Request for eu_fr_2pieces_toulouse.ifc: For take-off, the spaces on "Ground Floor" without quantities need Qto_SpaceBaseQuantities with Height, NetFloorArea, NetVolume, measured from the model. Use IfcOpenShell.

First a look at what the model holds.

```python
import ifcopenshell
import ifcopenshell.util.element
import ifcopenshell.util.unit

model = ifcopenshell.open("eu_fr_2pieces_toulouse.ifc")
print(model.schema)
for unit_type in ("LENGTHUNIT", "AREAUNIT", "VOLUMEUNIT"):
    print(unit_type, ifcopenshell.util.unit.calculate_unit_scale(model, unit_type))
storey = next(s for s in model.by_type("IfcBuildingStorey") if s.Name == "Ground Floor")
spaces = [e for e in ifcopenshell.util.element.get_decomposition(storey) if e.is_a("IfcSpace")]
for e in sorted(spaces, key=lambda e: e.id()):
    print(e.id(), e.is_a(), e.Name, list(ifcopenshell.util.element.get_psets(e, qtos_only=True)), sep=" | ")
```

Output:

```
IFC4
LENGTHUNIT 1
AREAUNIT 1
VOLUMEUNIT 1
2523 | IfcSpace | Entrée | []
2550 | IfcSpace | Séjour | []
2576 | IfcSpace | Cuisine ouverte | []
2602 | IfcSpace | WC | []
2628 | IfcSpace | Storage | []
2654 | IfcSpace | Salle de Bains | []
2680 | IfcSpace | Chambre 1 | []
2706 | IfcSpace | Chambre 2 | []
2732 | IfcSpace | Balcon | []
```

```python
import ifcopenshell
import ifcopenshell.api.pset
import ifcopenshell.geom
import ifcopenshell.util.element
import ifcopenshell.util.shape
import ifcopenshell.util.unit

model = ifcopenshell.open("eu_fr_2pieces_toulouse.ifc")
unit_scale = ifcopenshell.util.unit.calculate_unit_scale(model)
area_scale = ifcopenshell.util.unit.calculate_unit_scale(model, "AREAUNIT")
volume_scale = ifcopenshell.util.unit.calculate_unit_scale(model, "VOLUMEUNIT")
settings = ifcopenshell.geom.settings()

storey = next(s for s in model.by_type("IfcBuildingStorey") if s.Name == "Ground Floor")
spaces = [e for e in ifcopenshell.util.element.get_decomposition(storey) if e.is_a("IfcSpace")]

for e in sorted(spaces, key=lambda e: e.id()):
    if ifcopenshell.util.element.get_psets(e, qtos_only=True, should_inherit=False):
        continue
    # Geometry comes back in metres, in the element's own axes.
    shape = ifcopenshell.geom.create_shape(settings, e)
    values = {
        "Height": ifcopenshell.util.shape.get_z(shape.geometry) / unit_scale,
        "NetFloorArea": ifcopenshell.util.shape.get_footprint_area(shape.geometry) / area_scale,
        "NetVolume": ifcopenshell.util.shape.get_volume(shape.geometry) / volume_scale,
    }
    qto = ifcopenshell.api.pset.add_qto(model, product=e, name="Qto_SpaceBaseQuantities")
    ifcopenshell.api.pset.edit_qto(model, qto=qto, properties=values)
    print(e.id(), {k: round(v, 3) for k, v in values.items()})

model.write("eu_fr_2pieces_toulouse_updated.ifc")
```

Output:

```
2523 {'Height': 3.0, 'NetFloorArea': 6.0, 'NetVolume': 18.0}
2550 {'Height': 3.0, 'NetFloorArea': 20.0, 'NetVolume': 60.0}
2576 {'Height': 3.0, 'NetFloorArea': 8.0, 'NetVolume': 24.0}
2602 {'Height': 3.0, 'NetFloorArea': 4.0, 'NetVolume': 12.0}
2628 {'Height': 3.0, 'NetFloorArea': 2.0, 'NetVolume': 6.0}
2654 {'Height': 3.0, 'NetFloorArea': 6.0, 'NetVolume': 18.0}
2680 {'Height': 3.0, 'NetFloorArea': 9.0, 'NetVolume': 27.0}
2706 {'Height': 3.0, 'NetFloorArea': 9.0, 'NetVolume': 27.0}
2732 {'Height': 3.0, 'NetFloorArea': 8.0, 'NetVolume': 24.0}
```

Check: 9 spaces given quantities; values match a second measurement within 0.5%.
